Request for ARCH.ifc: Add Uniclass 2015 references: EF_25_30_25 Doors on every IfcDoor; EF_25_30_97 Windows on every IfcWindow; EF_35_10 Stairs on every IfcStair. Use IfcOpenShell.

First a look at what the model holds.

```python
import ifcopenshell

model = ifcopenshell.open("ARCH.ifc")
print(model.schema)
print("classifications:", [c.Name for c in model.by_type("IfcClassification")])
for ifc_class in ("IfcDoor", "IfcRoof", "IfcStair", "IfcWall", "IfcWindow"):
    print(ifc_class, len(model.by_type(ifc_class)))
```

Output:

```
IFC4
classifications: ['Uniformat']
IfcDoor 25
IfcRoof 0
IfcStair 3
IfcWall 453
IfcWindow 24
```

```python
import ifcopenshell
import ifcopenshell.api.classification

model = ifcopenshell.open("ARCH.ifc")

system = ifcopenshell.api.classification.add_classification(model, classification="Uniclass 2015")

codes = {
    "IfcDoor": ("EF_25_30_25", "Doors"),
    "IfcWindow": ("EF_25_30_97", "Windows"),
    "IfcStair": ("EF_35_10", "Stairs"),
}
for ifc_class, (code, name) in codes.items():
    products = model.by_type(ifc_class)
    ifcopenshell.api.classification.add_reference(
        model, products=products, classification=system, identification=code, name=name
    )
    print(code, len(products))

model.write("ARCH_updated.ifc")
```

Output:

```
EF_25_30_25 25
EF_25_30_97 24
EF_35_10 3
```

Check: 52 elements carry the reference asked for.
